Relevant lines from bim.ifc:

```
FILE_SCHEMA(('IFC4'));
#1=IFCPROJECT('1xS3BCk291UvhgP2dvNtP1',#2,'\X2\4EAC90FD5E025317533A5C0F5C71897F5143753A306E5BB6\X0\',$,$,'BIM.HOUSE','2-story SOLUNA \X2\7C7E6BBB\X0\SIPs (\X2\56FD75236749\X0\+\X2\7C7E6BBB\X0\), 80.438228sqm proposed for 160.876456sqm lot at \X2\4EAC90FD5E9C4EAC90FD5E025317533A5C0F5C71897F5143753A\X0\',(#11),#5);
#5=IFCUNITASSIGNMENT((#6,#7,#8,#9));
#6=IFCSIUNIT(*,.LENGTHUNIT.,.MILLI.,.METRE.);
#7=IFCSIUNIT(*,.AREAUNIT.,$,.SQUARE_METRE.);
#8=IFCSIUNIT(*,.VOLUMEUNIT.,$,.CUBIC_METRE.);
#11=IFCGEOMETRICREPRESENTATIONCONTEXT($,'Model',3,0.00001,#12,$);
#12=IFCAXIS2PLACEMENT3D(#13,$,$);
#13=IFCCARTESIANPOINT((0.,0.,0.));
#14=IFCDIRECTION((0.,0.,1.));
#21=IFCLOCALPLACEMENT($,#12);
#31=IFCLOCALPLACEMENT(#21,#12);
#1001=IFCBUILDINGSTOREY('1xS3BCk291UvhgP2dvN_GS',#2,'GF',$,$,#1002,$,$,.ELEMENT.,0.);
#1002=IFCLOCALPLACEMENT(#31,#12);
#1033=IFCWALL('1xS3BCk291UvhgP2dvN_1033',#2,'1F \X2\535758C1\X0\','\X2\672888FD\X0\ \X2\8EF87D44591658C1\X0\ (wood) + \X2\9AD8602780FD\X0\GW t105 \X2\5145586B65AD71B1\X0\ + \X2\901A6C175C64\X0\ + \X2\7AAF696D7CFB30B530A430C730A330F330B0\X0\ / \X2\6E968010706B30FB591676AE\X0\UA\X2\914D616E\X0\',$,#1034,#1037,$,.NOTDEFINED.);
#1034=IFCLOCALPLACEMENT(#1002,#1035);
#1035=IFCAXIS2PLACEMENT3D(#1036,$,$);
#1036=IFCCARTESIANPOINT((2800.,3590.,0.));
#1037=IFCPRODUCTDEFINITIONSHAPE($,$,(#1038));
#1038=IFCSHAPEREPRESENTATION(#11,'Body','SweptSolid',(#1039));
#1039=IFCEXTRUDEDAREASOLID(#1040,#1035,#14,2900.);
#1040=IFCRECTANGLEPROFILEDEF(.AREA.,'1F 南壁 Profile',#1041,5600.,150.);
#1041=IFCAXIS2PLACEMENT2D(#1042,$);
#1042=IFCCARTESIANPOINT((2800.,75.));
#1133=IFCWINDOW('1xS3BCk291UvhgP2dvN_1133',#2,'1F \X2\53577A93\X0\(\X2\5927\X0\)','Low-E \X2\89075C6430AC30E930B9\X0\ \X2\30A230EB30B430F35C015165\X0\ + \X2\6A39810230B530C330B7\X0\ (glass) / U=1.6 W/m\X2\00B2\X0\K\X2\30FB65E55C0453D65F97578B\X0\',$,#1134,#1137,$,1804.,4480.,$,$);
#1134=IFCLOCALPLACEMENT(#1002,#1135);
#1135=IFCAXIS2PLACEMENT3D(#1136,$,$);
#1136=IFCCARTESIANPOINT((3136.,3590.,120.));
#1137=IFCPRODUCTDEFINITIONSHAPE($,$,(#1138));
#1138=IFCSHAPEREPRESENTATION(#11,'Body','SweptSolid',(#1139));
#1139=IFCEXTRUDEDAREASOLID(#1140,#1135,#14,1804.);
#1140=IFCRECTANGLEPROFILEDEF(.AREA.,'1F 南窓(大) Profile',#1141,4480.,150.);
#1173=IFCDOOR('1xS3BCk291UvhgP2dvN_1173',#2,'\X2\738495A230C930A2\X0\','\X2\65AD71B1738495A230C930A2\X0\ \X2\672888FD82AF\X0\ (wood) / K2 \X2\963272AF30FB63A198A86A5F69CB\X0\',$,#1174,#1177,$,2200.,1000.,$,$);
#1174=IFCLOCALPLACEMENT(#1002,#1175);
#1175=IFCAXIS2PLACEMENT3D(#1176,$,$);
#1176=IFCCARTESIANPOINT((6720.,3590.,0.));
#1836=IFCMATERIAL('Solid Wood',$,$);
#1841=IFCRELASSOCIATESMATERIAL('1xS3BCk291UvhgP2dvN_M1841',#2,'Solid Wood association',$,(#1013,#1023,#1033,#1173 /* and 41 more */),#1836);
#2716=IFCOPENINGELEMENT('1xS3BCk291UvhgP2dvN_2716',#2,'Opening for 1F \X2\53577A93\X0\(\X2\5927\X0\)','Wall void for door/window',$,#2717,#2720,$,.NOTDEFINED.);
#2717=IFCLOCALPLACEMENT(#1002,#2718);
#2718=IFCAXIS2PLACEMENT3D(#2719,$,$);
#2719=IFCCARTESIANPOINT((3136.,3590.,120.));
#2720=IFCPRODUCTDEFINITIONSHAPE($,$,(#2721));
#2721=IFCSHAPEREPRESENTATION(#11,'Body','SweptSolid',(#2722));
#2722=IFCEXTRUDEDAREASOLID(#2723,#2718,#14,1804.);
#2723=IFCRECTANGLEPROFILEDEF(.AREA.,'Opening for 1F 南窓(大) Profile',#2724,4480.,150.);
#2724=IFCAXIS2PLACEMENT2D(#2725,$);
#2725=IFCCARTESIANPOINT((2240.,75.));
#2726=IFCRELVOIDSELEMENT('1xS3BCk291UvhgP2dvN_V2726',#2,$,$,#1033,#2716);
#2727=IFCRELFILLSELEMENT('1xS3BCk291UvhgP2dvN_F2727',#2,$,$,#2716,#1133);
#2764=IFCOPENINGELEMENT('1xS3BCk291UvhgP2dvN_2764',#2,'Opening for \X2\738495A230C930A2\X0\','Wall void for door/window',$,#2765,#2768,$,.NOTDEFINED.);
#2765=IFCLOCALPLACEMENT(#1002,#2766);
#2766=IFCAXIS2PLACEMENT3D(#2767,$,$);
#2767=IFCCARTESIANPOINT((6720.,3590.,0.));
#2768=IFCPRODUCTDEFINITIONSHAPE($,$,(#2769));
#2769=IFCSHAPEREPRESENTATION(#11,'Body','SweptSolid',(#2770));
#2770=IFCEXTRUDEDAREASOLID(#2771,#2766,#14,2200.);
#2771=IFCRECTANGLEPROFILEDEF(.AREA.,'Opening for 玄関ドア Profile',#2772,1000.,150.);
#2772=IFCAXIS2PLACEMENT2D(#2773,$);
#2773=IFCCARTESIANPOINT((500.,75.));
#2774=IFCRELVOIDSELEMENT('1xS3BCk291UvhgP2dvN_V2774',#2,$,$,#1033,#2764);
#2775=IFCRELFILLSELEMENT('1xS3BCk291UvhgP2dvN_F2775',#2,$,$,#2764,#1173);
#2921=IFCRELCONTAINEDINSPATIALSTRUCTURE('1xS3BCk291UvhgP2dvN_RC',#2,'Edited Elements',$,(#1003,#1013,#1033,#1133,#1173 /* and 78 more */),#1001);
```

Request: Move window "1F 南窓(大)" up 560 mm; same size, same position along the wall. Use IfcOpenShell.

```python
import numpy as np
import ifcopenshell
import ifcopenshell.api.geometry
import ifcopenshell.util.placement
import ifcopenshell.util.unit

model = ifcopenshell.open("bim.ifc")
unit_scale = ifcopenshell.util.unit.calculate_unit_scale(model)

window = model.by_id(1133)
opening = window.FillsVoids[0].RelatingOpeningElement
dz = 560.0

shift = np.array([0.0, 0.0, dz])
# The window is not placed relative to its opening, so move both.
for product in (opening, window):
    matrix = ifcopenshell.util.placement.get_local_placement(product.ObjectPlacement)
    matrix[:3, 3] += shift
    ifcopenshell.api.geometry.edit_object_placement(model, product=product, matrix=matrix, is_si=False)

print(f"moved by {dz * unit_scale:+.3f} m")

model.write("bim_v2.ifc")
```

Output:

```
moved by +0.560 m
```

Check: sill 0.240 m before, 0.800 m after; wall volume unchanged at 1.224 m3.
